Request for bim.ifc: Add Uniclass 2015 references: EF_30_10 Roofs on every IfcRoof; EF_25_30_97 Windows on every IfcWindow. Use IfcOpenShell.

First a look at what the model holds.

```python
import ifcopenshell

model = ifcopenshell.open("bim.ifc")
print(model.schema)
print("classifications:", [c.Name for c in model.by_type("IfcClassification")])
for ifc_class in ("IfcDoor", "IfcRoof", "IfcStair", "IfcWall", "IfcWindow"):
    print(ifc_class, len(model.by_type(ifc_class)))
```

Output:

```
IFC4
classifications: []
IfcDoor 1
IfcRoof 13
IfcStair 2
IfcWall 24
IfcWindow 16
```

```python
import ifcopenshell
import ifcopenshell.api.classification

model = ifcopenshell.open("bim.ifc")

system = ifcopenshell.api.classification.add_classification(model, classification="Uniclass 2015")

codes = {
    "IfcRoof": ("EF_30_10", "Roofs"),
    "IfcWindow": ("EF_25_30_97", "Windows"),
}
for ifc_class, (code, name) in codes.items():
    products = model.by_type(ifc_class)
    ifcopenshell.api.classification.add_reference(
        model, products=products, classification=system, identification=code, name=name
    )
    print(code, len(products))

model.write("bim-out.ifc")
```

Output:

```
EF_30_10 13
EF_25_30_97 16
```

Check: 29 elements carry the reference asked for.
